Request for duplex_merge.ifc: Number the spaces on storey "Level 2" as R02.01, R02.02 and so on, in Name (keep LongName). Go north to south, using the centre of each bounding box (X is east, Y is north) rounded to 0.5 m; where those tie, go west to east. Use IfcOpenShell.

First a look at what the model holds.

```python
import ifcopenshell
import ifcopenshell.util.element
import ifcopenshell.util.placement

model = ifcopenshell.open("duplex_merge.ifc")
print(model.schema)
storey = next(s for s in model.by_type("IfcBuildingStorey") if s.Name == "Level 2")
spaces = [e for e in ifcopenshell.util.element.get_decomposition(storey) if e.is_a("IfcSpace")]
for e in sorted(spaces, key=lambda e: e.id()):
    origin = ifcopenshell.util.placement.get_local_placement(e.ObjectPlacement)[:3, 3]
    print(e.id(), e.Name, e.LongName, origin.round(2) + 0.0, sep=" | ")
```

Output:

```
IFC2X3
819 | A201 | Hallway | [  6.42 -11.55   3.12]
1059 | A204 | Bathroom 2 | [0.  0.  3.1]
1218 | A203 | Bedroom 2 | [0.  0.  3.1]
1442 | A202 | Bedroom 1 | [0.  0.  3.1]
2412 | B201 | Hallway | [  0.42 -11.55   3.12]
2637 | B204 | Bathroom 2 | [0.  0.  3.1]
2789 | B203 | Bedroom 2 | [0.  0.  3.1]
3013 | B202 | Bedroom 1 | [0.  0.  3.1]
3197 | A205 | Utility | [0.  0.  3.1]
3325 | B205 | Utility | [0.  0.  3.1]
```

```python
import ifcopenshell
import ifcopenshell.geom
import ifcopenshell.util.element
import ifcopenshell.util.shape

model = ifcopenshell.open("duplex_merge.ifc")
settings = ifcopenshell.geom.settings()
settings.set("use-world-coords", True)


def centre(element):
    shape = ifcopenshell.geom.create_shape(settings, element)
    return ifcopenshell.util.shape.get_bbox_centroid(shape.geometry)


storey = next(s for s in model.by_type("IfcBuildingStorey") if s.Name == "Level 2")
spaces = [e for e in ifcopenshell.util.element.get_decomposition(storey) if e.is_a("IfcSpace")]

# Insertion points can sit at a corner or the storey origin, so sort by the geometry (in metres).
centres = {e: centre(e) for e in spaces}
spaces.sort(key=lambda e: (-round(centres[e][1] / 0.5), centres[e][0]))

for i, e in enumerate(spaces, start=1):
    number = f"R02.{i:02d}"
    e.Name = number
    print(e.id(), number)

model.write("duplex_merge_edited.ifc")
```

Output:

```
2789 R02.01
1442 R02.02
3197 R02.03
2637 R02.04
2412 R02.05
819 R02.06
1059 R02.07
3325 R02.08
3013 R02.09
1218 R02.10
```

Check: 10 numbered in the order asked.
